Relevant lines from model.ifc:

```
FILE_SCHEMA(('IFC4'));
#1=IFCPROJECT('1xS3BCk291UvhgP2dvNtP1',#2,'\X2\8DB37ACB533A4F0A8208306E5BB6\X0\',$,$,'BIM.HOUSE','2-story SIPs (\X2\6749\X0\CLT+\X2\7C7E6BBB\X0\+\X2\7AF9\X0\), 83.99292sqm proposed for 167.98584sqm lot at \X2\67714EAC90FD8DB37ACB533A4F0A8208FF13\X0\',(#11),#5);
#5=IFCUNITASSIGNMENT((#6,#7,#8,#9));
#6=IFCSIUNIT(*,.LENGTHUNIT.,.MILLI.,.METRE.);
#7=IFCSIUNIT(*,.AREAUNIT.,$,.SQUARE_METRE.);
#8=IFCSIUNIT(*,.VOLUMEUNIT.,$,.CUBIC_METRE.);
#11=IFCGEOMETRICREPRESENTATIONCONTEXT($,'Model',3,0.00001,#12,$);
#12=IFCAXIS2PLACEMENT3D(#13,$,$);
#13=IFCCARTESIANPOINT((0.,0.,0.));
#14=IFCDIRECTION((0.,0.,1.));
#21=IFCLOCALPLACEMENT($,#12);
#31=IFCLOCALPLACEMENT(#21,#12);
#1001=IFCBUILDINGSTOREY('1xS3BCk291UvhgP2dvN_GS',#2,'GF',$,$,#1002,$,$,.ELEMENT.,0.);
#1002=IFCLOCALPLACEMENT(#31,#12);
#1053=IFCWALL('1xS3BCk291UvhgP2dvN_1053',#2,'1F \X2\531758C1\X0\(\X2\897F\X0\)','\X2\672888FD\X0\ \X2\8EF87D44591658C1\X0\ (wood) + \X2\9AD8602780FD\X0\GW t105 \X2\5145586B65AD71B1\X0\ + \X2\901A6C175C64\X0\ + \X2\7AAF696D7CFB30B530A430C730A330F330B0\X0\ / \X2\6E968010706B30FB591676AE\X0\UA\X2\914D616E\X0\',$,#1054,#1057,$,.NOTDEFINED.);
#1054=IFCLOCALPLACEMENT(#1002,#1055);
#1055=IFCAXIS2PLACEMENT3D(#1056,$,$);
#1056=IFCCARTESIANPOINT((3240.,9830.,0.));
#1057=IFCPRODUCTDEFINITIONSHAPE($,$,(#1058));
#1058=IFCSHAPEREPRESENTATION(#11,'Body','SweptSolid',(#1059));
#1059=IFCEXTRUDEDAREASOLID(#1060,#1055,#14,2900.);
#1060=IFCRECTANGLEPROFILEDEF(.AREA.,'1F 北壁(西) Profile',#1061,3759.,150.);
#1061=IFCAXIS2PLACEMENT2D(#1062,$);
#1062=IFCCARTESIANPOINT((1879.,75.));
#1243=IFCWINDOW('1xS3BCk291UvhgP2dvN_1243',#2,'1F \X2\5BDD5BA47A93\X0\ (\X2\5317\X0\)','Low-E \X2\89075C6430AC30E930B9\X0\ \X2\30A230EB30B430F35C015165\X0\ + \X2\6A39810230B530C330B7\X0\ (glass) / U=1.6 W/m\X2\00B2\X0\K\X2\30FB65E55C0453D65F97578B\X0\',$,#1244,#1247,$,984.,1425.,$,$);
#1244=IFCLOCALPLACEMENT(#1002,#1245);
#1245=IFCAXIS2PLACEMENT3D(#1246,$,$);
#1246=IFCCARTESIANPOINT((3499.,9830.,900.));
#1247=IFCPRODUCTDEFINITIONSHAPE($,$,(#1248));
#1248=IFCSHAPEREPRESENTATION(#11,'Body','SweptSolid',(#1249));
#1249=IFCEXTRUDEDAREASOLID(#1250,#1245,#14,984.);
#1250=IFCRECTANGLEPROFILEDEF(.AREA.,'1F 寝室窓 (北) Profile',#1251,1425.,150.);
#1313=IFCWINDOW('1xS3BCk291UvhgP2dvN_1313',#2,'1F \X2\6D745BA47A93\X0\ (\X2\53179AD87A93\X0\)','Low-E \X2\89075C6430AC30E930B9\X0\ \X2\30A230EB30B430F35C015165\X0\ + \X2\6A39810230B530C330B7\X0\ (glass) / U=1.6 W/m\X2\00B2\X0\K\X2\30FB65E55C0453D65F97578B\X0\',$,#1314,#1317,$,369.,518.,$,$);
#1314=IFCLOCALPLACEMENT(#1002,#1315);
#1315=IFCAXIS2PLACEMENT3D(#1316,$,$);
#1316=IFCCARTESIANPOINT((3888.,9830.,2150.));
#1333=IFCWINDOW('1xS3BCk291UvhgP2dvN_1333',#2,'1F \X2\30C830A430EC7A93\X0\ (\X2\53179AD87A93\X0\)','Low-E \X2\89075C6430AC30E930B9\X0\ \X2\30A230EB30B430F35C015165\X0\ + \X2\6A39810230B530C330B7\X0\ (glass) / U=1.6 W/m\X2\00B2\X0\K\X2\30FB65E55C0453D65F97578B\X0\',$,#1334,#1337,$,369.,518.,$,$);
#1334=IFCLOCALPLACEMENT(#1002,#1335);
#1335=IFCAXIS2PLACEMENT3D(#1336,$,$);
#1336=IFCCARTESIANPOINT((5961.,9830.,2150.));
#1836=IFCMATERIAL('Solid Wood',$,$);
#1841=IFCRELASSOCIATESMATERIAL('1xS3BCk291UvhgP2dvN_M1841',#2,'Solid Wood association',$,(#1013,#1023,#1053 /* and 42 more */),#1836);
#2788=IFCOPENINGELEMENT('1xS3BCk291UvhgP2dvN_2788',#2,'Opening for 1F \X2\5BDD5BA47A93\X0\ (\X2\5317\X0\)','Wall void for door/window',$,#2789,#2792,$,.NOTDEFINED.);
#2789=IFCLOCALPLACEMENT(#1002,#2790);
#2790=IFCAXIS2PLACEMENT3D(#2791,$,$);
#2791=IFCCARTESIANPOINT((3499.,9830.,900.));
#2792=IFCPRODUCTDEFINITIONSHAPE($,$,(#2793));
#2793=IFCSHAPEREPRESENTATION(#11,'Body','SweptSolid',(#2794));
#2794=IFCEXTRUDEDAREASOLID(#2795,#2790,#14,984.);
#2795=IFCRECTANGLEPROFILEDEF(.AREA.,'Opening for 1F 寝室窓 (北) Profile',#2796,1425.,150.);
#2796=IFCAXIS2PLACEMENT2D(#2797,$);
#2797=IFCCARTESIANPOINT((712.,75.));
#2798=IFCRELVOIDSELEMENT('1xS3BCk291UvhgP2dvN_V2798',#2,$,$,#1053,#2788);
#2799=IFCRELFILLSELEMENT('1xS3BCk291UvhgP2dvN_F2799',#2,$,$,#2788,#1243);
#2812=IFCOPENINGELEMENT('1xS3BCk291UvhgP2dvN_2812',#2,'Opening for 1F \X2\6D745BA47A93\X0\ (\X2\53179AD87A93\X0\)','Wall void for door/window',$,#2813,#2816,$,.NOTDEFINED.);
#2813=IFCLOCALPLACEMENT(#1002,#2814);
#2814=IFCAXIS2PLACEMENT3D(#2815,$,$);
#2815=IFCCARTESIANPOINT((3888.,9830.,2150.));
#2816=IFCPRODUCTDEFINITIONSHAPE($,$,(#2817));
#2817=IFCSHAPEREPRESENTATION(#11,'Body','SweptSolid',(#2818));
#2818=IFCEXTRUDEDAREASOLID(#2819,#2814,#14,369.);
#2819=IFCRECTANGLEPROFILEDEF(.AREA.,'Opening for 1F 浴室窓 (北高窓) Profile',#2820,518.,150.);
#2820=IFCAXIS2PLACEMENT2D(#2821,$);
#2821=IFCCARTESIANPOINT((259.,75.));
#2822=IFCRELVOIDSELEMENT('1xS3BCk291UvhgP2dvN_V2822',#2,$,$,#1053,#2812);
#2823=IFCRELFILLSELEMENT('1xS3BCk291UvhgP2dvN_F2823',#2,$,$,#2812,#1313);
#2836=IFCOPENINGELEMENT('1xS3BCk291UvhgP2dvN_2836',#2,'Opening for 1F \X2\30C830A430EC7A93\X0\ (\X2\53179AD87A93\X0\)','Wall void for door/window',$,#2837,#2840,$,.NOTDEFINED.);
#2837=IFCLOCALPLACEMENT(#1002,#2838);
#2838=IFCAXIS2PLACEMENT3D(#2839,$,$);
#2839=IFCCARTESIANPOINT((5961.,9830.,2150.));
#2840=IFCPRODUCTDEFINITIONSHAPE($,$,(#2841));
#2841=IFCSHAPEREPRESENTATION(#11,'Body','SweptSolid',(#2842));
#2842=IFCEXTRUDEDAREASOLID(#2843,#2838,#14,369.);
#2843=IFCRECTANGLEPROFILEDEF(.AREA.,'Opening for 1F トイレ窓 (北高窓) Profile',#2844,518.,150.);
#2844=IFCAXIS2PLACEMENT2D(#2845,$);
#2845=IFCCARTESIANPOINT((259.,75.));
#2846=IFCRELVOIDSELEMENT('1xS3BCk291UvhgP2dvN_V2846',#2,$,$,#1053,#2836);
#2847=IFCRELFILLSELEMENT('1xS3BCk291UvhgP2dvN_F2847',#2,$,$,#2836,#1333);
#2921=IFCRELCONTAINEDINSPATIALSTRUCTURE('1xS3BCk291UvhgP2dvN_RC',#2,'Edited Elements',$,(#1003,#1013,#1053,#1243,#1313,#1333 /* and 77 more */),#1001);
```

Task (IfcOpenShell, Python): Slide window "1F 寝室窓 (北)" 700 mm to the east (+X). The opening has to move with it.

```python
import ifcopenshell
import ifcopenshell.api.geometry
import ifcopenshell.util.placement
import ifcopenshell.util.unit

model = ifcopenshell.open("model.ifc")
unit_scale = ifcopenshell.util.unit.calculate_unit_scale(model)

window = model.by_id(1243)
opening = window.FillsVoids[0].RelatingOpeningElement
wall = opening.VoidsElements[0].RelatingBuildingElement

wall_matrix = ifcopenshell.util.placement.get_local_placement(wall.ObjectPlacement)
shift = wall_matrix[:3, 0] * 0.7 / unit_scale
before = ifcopenshell.util.placement.get_local_placement(window.ObjectPlacement)[:3, 3].copy()

# The window is not placed relative to its opening, so move both.
for product in (opening, window):
    matrix = ifcopenshell.util.placement.get_local_placement(product.ObjectPlacement)
    matrix[:3, 3] += shift
    ifcopenshell.api.geometry.edit_object_placement(model, product=product, matrix=matrix, is_si=False)

after = ifcopenshell.util.placement.get_local_placement(window.ObjectPlacement)[:3, 3]
print("window moved by", (after - before).round(3) + 0.0)

model.write("model_updated.ifc")
```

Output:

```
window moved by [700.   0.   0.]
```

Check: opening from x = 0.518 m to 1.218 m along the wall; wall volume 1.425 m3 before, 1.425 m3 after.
